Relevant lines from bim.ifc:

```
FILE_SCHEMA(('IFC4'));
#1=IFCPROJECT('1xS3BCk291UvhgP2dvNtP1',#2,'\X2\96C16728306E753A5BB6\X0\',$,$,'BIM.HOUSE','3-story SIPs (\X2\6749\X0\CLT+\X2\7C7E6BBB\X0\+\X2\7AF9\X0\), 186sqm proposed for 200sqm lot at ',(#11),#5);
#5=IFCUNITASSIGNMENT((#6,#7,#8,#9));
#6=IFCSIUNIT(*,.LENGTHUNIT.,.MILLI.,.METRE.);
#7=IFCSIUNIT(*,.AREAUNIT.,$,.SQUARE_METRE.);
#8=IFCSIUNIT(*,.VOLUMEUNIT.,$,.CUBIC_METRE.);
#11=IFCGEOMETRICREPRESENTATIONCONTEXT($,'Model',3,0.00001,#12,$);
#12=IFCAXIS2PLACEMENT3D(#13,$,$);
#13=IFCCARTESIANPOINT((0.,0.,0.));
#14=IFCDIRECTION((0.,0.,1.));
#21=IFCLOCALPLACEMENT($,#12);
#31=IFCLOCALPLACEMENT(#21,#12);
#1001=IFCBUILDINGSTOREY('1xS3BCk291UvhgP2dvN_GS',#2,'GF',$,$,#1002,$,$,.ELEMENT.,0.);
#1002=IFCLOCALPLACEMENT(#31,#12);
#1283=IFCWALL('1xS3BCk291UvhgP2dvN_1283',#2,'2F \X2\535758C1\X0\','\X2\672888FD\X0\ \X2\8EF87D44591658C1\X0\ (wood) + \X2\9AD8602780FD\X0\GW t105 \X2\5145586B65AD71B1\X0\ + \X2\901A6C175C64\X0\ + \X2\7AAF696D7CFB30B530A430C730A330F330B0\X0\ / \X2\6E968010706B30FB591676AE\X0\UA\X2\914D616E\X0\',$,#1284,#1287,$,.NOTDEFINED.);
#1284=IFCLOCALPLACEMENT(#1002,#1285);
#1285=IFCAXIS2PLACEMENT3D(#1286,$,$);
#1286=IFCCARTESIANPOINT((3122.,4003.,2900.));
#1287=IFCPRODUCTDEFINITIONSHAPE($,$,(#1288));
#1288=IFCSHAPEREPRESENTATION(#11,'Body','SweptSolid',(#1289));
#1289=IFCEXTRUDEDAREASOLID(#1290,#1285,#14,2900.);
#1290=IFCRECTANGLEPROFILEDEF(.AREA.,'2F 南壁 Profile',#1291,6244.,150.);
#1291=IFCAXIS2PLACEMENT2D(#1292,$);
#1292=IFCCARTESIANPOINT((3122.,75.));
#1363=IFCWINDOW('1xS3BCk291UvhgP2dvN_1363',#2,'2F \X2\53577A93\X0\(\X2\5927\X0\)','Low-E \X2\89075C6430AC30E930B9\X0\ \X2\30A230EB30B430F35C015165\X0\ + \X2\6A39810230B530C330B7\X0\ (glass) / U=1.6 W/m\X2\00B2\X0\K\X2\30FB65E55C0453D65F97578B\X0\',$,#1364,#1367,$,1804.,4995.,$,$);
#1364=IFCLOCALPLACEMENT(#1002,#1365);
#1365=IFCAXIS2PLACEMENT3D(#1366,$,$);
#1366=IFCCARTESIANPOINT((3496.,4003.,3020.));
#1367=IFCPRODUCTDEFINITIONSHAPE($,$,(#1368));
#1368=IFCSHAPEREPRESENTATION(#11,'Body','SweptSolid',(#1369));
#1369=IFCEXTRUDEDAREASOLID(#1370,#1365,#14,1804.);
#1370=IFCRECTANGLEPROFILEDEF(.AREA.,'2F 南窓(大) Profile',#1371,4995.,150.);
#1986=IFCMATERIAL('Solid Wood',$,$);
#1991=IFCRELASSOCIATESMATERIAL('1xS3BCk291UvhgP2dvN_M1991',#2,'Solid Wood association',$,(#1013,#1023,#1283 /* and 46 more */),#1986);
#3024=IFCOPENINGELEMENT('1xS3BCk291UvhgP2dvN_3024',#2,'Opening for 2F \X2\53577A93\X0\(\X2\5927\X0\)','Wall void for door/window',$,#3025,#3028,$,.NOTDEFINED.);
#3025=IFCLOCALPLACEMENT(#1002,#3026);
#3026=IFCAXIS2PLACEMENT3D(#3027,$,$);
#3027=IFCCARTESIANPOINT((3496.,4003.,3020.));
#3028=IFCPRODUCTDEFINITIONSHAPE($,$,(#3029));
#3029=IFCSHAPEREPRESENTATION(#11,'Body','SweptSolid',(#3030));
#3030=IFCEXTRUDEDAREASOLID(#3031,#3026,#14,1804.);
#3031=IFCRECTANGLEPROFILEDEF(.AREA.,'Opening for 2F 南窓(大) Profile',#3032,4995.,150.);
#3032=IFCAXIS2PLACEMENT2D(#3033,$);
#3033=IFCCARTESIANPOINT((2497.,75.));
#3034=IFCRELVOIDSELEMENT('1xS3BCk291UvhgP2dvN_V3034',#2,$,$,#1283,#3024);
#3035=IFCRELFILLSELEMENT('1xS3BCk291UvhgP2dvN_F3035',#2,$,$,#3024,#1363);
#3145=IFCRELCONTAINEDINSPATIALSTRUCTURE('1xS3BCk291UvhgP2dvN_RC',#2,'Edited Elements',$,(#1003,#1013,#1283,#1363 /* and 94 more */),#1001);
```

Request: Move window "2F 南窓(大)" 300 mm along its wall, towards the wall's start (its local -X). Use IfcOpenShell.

```python
import ifcopenshell
import ifcopenshell.api.geometry
import ifcopenshell.util.placement

model = ifcopenshell.open("bim.ifc")

window = model.by_guid("1xS3BCk291UvhgP2dvN_1363")
opening = window.FillsVoids[0].RelatingOpeningElement
wall = opening.VoidsElements[0].RelatingBuildingElement

wall_matrix = ifcopenshell.util.placement.get_local_placement(wall.ObjectPlacement)
shift = wall_matrix[:3, 0] * -300.0
before = ifcopenshell.util.placement.get_local_placement(window.ObjectPlacement)[:3, 3].copy()

# The window is not placed relative to its opening, so move both.
for product in (opening, window):
    matrix = ifcopenshell.util.placement.get_local_placement(product.ObjectPlacement)
    matrix[:3, 3] += shift
    ifcopenshell.api.geometry.edit_object_placement(model, product=product, matrix=matrix, is_si=False)

after = ifcopenshell.util.placement.get_local_placement(window.ObjectPlacement)[:3, 3]
print("window moved by", (after - before).round(3) + 0.0)

model.write("bim_edited.ifc")
```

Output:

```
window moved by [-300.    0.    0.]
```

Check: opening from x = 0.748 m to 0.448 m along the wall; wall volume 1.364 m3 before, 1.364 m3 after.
